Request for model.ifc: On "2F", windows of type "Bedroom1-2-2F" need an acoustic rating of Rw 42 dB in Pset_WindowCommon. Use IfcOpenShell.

First a look at what the model holds.

```python
import ifcopenshell
import ifcopenshell.util.element

model = ifcopenshell.open("model.ifc")
print(model.schema)
storey = next(s for s in model.by_type("IfcBuildingStorey") if s.Name == "2F")
windows = [e for e in ifcopenshell.util.element.get_decomposition(storey) if e.is_a("IfcWindow")]
seen = {}
for e in windows:
    element_type = ifcopenshell.util.element.get_type(e)
    key = (element_type.Name if element_type != e and element_type else None, ifcopenshell.util.element.get_pset(e, "Pset_WindowCommon", "AcousticRating"))
    seen[key] = seen.get(key, 0) + 1
for (name, value), count in sorted(seen.items(), key=str):
    print(count, "x", name, "|", value)
```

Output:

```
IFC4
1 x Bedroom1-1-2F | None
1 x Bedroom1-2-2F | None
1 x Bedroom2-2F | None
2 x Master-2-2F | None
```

```python
import ifcopenshell
import ifcopenshell.api.pset
import ifcopenshell.util.element

model = ifcopenshell.open("model.ifc")

storey = next(s for s in model.by_type("IfcBuildingStorey") if s.Name == "2F")
windows = [e for e in ifcopenshell.util.element.get_decomposition(storey) if e.is_a("IfcWindow")]

count = 0
for e in windows:
    element_type = ifcopenshell.util.element.get_type(e)
    if element_type in (None, e) or element_type.Name != "Bedroom1-2-2F":
        continue
    # add_pset returns the element's existing set when there is one.
    pset = ifcopenshell.api.pset.add_pset(model, product=e, name="Pset_WindowCommon")
    ifcopenshell.api.pset.edit_pset(model, pset=pset, properties={"AcousticRating": "Rw 42 dB"})
    count += 1

print(count, "windows updated")

model.write("model_v2.ifc")
```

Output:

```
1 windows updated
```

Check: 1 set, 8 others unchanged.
